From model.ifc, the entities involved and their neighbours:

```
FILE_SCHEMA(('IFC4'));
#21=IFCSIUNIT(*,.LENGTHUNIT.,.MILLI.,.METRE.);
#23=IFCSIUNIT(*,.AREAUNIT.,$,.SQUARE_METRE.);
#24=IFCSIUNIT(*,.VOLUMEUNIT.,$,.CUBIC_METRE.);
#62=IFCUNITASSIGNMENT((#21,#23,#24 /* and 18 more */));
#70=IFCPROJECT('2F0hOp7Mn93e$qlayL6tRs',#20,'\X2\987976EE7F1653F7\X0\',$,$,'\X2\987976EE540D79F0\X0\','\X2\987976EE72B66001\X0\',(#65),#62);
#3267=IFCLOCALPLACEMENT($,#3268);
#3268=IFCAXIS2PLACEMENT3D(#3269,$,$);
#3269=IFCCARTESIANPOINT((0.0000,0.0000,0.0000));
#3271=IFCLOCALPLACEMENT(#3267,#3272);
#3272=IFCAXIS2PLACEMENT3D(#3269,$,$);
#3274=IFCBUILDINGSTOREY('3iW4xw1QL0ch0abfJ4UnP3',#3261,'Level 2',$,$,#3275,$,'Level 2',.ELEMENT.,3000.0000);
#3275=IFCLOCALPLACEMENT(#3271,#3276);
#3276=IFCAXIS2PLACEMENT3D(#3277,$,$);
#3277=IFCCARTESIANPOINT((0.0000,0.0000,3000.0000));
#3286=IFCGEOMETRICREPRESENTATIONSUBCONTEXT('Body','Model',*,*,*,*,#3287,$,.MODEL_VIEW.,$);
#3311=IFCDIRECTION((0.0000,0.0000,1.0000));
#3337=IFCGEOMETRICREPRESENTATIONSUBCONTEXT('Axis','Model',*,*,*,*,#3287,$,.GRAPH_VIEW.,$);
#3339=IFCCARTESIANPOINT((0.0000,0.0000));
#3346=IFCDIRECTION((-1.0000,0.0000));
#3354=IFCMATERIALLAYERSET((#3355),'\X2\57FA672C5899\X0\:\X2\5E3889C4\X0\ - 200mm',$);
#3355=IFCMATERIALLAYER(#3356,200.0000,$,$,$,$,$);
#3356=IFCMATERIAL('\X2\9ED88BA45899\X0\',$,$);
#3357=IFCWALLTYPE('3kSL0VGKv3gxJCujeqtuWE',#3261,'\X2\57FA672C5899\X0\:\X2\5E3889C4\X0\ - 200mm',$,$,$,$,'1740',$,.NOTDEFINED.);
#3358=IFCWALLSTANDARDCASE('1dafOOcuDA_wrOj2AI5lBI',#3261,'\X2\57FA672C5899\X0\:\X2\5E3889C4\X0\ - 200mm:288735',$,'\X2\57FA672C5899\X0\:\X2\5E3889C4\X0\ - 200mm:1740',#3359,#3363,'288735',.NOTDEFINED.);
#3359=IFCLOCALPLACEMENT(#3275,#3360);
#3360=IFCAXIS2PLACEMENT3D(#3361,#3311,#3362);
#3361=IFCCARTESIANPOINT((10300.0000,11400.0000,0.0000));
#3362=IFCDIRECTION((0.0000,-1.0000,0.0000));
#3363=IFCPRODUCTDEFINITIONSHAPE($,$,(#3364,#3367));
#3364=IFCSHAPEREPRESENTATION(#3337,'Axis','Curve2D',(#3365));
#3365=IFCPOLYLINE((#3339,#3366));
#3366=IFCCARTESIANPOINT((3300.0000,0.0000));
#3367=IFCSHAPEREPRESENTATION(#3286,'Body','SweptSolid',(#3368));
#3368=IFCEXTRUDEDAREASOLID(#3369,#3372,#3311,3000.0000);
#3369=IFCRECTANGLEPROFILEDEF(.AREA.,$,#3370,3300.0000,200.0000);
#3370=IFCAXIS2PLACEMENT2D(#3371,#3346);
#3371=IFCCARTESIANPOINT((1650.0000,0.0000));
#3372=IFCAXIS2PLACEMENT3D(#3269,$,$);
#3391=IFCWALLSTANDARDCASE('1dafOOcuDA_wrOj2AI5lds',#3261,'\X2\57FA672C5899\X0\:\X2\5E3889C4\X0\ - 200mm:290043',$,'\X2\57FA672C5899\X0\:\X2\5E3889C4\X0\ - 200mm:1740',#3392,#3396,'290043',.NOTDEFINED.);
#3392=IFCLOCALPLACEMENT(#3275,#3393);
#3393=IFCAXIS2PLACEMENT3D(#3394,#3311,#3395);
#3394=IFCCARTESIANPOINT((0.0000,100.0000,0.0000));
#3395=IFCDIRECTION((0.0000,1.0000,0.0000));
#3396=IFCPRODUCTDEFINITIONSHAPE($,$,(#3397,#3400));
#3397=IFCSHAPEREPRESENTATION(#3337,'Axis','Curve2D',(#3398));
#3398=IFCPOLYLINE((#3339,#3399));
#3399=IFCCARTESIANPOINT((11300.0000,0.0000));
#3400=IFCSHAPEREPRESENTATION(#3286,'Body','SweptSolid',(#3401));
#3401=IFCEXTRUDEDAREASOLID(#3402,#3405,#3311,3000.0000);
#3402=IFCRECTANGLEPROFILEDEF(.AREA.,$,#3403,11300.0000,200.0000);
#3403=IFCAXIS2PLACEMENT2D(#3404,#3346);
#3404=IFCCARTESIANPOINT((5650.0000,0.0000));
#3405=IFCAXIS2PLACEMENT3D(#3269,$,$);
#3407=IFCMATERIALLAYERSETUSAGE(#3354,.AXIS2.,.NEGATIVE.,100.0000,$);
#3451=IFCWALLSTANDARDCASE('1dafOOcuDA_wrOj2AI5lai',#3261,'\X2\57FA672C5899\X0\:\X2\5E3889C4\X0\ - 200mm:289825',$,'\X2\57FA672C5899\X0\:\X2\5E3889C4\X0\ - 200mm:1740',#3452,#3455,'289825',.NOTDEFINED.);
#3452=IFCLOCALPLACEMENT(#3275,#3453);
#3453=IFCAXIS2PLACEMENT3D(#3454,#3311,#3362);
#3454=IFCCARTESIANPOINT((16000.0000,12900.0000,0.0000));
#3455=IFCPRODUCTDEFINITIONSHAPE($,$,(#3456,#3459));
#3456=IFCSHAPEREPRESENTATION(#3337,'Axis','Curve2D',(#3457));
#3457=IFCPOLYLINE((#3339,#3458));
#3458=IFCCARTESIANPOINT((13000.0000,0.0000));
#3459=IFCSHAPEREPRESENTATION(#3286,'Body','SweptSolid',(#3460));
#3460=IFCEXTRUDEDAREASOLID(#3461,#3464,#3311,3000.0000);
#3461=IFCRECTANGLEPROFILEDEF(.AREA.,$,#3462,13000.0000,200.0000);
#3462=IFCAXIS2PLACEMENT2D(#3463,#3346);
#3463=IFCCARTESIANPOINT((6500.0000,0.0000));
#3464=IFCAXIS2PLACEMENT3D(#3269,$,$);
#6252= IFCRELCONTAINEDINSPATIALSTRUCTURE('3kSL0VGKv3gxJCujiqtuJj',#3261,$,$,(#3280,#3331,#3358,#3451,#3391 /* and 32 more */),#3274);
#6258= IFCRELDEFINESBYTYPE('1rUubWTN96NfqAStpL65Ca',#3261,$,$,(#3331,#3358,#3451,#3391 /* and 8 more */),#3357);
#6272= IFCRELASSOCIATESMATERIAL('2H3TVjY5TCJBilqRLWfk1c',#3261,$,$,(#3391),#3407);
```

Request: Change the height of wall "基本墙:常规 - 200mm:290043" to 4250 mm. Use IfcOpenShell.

```python
import ifcopenshell
import ifcopenshell.geom
import ifcopenshell.util.representation
import ifcopenshell.util.shape
import ifcopenshell.util.unit

model = ifcopenshell.open("model.ifc")
unit_scale = ifcopenshell.util.unit.calculate_unit_scale(model)
settings = ifcopenshell.geom.settings()


def volume(element):
    """Net volume in cubic metres, openings subtracted."""
    shape = ifcopenshell.geom.create_shape(settings, element)
    return ifcopenshell.util.shape.get_volume(shape.geometry)


wall = model.by_guid("1dafOOcuDA_wrOj2AI5lds")
before = volume(wall)

body = ifcopenshell.util.representation.get_representation(wall, "Model", "Body")
solid = body.Items[0]
old_height = solid.Depth
solid.Depth = 4.25 / unit_scale
after = volume(wall)

print(f"height {old_height:g} -> {solid.Depth:g}, volume {before:.3f} -> {after:.3f} m3")

model.write("model_rev.ifc")
```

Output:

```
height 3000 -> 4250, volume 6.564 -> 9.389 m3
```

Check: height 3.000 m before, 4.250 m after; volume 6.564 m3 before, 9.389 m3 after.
